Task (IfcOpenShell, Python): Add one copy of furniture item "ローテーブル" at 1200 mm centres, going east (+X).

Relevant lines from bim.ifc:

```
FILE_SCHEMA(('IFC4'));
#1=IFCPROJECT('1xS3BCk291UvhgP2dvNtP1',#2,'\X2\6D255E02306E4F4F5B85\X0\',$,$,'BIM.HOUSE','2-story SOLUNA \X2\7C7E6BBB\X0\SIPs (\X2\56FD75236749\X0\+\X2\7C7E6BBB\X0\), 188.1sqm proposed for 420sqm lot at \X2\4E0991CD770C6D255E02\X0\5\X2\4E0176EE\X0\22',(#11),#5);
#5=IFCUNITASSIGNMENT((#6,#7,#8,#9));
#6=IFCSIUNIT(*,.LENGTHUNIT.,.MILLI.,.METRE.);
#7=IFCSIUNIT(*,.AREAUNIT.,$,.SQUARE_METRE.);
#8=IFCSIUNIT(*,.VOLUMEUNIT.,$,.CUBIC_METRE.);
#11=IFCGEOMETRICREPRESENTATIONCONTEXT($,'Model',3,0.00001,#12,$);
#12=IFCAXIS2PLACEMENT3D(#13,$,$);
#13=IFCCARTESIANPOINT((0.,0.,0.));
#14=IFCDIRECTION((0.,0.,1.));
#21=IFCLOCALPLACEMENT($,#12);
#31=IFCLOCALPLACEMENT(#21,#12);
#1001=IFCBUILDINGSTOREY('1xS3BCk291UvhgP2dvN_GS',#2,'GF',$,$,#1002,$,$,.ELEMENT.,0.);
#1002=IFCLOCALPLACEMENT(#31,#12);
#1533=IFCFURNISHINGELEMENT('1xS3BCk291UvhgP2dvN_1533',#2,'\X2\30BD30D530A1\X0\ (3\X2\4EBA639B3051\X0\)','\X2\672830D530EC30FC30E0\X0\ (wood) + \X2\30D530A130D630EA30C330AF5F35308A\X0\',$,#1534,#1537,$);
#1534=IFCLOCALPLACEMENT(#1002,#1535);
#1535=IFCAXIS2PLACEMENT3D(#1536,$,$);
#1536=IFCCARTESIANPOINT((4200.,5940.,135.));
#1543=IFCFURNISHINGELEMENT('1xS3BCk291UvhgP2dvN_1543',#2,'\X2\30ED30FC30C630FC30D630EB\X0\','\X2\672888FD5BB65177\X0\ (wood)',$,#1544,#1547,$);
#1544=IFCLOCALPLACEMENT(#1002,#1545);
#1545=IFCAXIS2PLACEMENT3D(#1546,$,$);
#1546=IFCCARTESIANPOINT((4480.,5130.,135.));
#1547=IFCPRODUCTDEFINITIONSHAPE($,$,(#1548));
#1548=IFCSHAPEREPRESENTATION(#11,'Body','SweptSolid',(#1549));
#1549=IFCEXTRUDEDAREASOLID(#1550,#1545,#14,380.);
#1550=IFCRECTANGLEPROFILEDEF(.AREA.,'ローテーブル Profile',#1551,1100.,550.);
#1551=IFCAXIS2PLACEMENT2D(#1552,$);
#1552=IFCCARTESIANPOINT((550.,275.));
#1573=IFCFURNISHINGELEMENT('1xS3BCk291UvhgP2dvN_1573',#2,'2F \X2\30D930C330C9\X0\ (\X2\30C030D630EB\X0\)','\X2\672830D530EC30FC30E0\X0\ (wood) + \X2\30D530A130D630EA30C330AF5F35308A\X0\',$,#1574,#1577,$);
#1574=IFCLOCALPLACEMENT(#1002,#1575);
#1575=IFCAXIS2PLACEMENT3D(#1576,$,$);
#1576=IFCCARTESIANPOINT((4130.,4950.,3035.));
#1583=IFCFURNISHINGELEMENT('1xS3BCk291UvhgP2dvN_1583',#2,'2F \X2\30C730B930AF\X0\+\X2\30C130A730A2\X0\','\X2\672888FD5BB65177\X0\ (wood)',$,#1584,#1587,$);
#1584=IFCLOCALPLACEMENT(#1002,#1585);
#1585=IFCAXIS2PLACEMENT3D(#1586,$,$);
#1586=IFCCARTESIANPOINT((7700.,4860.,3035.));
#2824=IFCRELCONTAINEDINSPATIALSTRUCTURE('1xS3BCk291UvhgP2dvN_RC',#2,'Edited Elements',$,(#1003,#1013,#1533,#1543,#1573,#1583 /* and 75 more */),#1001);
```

```python
import numpy as np
import ifcopenshell
import ifcopenshell.api.geometry
import ifcopenshell.api.root
import ifcopenshell.util.element
import ifcopenshell.util.placement

model = ifcopenshell.open("bim.ifc")


def reuse_history(source, copy):
    """copy_class also copies each property set's owner history, people and application; keep the originals."""
    for rel in copy.IsDefinedBy:
        if rel.is_a("IfcRelDefinesByProperties") and (history := rel.RelatingPropertyDefinition.OwnerHistory):
            rel.RelatingPropertyDefinition.OwnerHistory = source.OwnerHistory
            ifcopenshell.util.element.remove_deep2(model, history)


source = model.by_guid("1xS3BCk291UvhgP2dvN_1543")
base = ifcopenshell.util.placement.get_local_placement(source.ObjectPlacement)
step = np.array([1.0, 0.0, 0.0]) * 1200.0

for i in range(1, 2):
    copy = ifcopenshell.api.root.copy_class(model, product=source)
    copy.Representation = ifcopenshell.util.element.copy_deep(
        model, source.Representation, exclude=["IfcGeometricRepresentationContext", "IfcRepresentationMap"]
    )
    reuse_history(source, copy)
    matrix = base.copy()
    matrix[:3, 3] += i * step
    print("added at", matrix[:3, 3].round(3) + 0.0)
    ifcopenshell.api.geometry.edit_object_placement(model, product=copy, matrix=matrix, is_si=False)

model.write("bim_rev.ifc")
```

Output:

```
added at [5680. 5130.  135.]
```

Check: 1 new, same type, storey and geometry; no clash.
